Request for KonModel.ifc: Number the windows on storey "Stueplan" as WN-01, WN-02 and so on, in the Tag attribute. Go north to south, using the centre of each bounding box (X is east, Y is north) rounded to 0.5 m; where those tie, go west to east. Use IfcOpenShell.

First a look at what the model holds.

```python
import ifcopenshell
import ifcopenshell.util.element
import ifcopenshell.util.placement

model = ifcopenshell.open("KonModel.ifc")
print(model.schema)
storey = next(s for s in model.by_type("IfcBuildingStorey") if s.Name == "Stueplan")
windows = [e for e in ifcopenshell.util.element.get_decomposition(storey) if e.is_a("IfcWindow")]
for e in sorted(windows, key=lambda e: e.id()):
    origin = ifcopenshell.util.placement.get_local_placement(e.ObjectPlacement)[:3, 3]
    print(e.id(), e.Tag, e.Name, origin.round(2) + 0.0, sep=" | ")
```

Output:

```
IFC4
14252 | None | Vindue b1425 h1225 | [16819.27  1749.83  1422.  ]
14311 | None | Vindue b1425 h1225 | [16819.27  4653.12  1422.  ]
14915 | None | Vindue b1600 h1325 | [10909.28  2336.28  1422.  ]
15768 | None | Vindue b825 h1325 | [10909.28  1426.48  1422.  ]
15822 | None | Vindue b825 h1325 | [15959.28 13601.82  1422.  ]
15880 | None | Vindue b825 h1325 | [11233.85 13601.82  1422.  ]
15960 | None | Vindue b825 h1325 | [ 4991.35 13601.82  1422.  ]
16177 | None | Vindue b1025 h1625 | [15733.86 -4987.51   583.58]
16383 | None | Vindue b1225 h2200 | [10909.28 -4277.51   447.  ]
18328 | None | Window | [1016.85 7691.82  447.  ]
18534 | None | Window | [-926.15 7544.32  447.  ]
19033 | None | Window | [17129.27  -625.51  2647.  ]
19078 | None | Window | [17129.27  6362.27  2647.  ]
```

```python
import ifcopenshell
import ifcopenshell.geom
import ifcopenshell.util.element
import ifcopenshell.util.shape

model = ifcopenshell.open("KonModel.ifc")
settings = ifcopenshell.geom.settings()
settings.set("use-world-coords", True)


def centre(element):
    shape = ifcopenshell.geom.create_shape(settings, element)
    return ifcopenshell.util.shape.get_bbox_centroid(shape.geometry)


storey = next(s for s in model.by_type("IfcBuildingStorey") if s.Name == "Stueplan")
windows = [e for e in ifcopenshell.util.element.get_decomposition(storey) if e.is_a("IfcWindow")]

# Insertion points can sit at a corner or the storey origin, so sort by the geometry (in metres).
centres = {e: centre(e) for e in windows}
windows.sort(key=lambda e: (-round(centres[e][1] / 0.5), centres[e][0]))

for i, e in enumerate(windows, start=1):
    number = f"WN-{i:02d}"
    e.Tag = number
    print(e.id(), number)

model.write("KonModel_updated.ifc")
```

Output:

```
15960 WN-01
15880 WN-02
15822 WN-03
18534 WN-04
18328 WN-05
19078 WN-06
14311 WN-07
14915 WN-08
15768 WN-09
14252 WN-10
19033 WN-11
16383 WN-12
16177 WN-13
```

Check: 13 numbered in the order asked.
